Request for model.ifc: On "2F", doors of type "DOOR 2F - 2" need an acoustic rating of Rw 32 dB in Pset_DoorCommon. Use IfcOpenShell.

First a look at what the model holds.

```python
import ifcopenshell
import ifcopenshell.util.element

model = ifcopenshell.open("model.ifc")
print(model.schema)
storey = next(s for s in model.by_type("IfcBuildingStorey") if s.Name == "2F")
doors = [e for e in ifcopenshell.util.element.get_decomposition(storey) if e.is_a("IfcDoor")]
seen = {}
for e in doors:
    element_type = ifcopenshell.util.element.get_type(e)
    key = (element_type.Name if element_type != e and element_type else None, ifcopenshell.util.element.get_pset(e, "Pset_DoorCommon", "AcousticRating"))
    seen[key] = seen.get(key, 0) + 1
for (name, value), count in sorted(seen.items(), key=str):
    print(count, "x", name, "|", value)
```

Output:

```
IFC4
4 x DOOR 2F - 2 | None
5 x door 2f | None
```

```python
import ifcopenshell
import ifcopenshell.api.pset
import ifcopenshell.util.element

model = ifcopenshell.open("model.ifc")

storey = next(s for s in model.by_type("IfcBuildingStorey") if s.Name == "2F")
doors = [e for e in ifcopenshell.util.element.get_decomposition(storey) if e.is_a("IfcDoor")]

count = 0
for e in doors:
    element_type = ifcopenshell.util.element.get_type(e)
    if element_type in (None, e) or element_type.Name != "DOOR 2F - 2":
        continue
    # add_pset returns the element's existing set when there is one.
    pset = ifcopenshell.api.pset.add_pset(model, product=e, name="Pset_DoorCommon")
    ifcopenshell.api.pset.edit_pset(model, pset=pset, properties={"AcousticRating": "Rw 32 dB"})
    count += 1

print(count, "doors updated")

model.write("model_v2.ifc")
```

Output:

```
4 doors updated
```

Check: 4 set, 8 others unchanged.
